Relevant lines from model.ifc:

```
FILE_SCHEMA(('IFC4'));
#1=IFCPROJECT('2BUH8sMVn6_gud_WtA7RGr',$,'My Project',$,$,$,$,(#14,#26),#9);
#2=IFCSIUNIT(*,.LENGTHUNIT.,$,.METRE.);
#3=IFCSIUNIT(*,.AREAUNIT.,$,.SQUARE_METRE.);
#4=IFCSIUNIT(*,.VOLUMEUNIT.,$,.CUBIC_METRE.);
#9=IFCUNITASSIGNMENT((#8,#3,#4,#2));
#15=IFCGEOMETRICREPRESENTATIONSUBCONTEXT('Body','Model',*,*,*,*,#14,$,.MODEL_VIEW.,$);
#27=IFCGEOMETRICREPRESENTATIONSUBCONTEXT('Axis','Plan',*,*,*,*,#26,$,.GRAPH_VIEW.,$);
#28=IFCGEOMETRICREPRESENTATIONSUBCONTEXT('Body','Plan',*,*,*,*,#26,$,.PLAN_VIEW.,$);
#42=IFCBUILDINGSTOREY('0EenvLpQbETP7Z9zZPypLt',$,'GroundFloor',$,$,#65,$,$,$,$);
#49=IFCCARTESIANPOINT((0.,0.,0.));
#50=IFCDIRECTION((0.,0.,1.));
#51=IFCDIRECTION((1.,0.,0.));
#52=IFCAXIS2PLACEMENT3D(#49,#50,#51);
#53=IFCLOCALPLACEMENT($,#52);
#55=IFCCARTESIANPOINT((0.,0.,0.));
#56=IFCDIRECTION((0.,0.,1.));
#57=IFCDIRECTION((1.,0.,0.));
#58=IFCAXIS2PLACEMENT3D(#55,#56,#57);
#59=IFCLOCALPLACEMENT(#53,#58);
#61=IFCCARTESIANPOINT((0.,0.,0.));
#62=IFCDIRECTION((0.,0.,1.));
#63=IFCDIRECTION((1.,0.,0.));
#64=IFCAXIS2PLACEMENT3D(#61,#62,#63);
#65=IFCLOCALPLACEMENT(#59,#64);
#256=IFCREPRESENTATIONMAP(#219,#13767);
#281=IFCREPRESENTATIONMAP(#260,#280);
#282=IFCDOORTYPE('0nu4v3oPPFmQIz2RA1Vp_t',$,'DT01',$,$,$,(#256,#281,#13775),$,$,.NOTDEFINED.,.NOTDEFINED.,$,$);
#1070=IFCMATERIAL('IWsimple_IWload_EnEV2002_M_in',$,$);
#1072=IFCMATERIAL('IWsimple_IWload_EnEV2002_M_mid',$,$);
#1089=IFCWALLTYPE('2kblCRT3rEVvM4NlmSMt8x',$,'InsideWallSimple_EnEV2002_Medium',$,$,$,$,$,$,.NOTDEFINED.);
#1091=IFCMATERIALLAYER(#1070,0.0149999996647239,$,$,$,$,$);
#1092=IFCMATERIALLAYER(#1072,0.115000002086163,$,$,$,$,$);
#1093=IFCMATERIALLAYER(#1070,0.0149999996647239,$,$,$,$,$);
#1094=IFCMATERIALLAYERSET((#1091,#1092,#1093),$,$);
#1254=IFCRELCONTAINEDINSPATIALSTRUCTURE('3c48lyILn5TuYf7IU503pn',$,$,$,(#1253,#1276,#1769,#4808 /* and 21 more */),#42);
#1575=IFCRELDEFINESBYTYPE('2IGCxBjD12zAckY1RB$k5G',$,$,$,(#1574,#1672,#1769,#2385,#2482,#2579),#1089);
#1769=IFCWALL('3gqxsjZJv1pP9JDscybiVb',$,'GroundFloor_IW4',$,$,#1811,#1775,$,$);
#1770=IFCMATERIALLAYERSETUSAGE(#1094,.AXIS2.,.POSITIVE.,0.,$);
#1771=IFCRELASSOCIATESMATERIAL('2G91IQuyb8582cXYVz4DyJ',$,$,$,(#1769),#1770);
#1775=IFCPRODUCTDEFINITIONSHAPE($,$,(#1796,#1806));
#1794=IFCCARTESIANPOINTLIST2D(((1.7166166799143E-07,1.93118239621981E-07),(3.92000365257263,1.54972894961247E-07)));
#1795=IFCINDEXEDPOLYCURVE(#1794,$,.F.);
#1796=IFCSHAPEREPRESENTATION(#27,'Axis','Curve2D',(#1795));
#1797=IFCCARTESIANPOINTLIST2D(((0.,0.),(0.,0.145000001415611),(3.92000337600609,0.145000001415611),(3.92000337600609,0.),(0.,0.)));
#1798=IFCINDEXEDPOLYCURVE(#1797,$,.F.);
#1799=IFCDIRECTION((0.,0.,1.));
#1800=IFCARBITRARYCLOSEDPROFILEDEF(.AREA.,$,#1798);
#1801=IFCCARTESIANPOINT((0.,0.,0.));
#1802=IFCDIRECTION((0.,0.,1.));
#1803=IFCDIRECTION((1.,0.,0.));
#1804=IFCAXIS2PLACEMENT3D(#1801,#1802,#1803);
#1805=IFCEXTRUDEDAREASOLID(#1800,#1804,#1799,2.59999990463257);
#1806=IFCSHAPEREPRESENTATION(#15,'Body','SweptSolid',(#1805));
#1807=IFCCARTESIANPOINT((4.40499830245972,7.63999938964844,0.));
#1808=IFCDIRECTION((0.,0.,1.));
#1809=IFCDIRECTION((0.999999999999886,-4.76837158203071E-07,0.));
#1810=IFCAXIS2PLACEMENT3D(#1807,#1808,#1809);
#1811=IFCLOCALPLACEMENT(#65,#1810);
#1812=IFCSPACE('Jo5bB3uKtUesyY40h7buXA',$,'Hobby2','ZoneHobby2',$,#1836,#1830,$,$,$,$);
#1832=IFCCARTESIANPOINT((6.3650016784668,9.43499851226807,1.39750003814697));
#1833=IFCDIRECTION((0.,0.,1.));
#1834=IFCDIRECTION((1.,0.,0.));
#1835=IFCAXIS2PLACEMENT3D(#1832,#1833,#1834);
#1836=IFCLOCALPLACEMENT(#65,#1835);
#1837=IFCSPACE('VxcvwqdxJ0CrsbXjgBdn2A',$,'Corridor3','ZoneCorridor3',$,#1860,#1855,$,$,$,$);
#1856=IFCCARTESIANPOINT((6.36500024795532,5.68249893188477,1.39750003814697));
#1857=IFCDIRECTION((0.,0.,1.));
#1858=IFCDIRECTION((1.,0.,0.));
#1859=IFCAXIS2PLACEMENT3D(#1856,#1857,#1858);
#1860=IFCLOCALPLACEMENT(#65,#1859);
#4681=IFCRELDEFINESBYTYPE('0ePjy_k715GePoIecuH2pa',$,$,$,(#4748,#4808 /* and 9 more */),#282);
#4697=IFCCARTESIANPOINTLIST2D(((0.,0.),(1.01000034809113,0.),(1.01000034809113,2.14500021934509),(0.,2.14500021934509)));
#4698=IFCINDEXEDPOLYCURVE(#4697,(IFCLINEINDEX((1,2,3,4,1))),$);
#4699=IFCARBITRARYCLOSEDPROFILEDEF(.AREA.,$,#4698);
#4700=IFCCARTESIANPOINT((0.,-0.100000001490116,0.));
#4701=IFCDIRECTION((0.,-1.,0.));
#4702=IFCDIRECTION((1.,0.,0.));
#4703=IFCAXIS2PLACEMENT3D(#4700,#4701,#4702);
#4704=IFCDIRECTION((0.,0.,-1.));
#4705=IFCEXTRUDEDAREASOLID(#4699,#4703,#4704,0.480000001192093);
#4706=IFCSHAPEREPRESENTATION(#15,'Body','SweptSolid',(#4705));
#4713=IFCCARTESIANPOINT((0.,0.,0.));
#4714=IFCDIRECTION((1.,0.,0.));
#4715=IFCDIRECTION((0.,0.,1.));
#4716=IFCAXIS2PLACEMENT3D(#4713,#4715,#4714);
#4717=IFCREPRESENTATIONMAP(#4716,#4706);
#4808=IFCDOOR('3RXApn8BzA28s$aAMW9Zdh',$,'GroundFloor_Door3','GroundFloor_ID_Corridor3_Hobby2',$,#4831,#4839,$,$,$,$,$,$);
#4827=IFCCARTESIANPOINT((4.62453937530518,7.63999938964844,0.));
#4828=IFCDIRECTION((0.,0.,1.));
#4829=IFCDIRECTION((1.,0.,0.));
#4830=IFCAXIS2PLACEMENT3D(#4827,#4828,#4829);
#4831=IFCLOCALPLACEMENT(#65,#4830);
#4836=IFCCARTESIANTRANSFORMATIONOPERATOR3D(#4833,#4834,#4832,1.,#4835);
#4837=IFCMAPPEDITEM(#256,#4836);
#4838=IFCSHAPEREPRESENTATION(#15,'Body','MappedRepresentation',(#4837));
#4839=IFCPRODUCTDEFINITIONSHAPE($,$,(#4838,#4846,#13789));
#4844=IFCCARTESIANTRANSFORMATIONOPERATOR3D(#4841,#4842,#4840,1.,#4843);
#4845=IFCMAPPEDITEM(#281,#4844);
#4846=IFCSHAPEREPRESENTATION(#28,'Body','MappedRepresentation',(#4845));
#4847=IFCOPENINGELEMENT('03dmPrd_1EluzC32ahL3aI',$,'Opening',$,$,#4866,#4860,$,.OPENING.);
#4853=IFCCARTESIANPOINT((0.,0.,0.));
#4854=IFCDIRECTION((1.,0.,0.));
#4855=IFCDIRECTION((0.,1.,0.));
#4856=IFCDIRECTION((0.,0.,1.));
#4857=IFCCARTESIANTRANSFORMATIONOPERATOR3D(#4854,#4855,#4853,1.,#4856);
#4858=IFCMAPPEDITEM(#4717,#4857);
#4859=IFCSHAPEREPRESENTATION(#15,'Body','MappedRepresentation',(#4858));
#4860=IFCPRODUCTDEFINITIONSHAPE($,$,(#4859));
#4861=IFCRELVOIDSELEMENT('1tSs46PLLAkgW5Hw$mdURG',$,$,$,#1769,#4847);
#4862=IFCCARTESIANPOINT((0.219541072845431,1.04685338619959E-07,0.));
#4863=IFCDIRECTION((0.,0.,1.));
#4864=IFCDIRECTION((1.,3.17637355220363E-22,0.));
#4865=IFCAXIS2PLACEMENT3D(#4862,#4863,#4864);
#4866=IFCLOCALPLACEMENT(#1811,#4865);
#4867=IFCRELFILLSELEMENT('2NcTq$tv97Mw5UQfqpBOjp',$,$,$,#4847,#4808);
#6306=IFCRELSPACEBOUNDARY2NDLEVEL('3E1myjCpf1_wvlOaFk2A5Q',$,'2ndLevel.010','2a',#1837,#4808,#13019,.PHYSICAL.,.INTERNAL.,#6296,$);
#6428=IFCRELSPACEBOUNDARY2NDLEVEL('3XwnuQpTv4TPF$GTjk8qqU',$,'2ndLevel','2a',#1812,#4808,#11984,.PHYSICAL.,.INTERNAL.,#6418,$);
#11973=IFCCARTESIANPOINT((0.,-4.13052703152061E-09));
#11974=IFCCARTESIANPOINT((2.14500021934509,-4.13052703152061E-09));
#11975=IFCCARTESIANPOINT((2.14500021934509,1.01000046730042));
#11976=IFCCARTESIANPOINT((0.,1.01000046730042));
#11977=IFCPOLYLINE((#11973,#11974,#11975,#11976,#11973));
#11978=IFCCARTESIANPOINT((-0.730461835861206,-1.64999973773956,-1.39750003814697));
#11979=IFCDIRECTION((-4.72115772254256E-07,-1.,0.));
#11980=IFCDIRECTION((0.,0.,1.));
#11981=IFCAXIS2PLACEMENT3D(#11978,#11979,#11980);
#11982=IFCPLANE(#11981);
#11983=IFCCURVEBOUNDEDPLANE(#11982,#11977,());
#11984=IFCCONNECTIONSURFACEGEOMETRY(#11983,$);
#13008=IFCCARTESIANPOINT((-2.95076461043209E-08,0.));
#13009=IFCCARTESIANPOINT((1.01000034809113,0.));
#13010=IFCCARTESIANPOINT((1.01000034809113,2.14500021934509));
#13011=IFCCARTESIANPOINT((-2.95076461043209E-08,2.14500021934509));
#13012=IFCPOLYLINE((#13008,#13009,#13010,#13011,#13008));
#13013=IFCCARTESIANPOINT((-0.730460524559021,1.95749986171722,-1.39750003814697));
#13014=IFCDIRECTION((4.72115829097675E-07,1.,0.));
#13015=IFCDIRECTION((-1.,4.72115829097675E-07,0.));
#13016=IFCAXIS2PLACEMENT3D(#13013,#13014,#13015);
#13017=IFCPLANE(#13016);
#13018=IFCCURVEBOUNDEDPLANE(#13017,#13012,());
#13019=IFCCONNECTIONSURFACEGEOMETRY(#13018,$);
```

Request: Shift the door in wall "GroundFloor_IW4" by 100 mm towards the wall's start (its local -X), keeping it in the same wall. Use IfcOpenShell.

```python
import numpy as np
import ifcopenshell
import ifcopenshell.api.geometry
import ifcopenshell.util.placement

model = ifcopenshell.open("model.ifc")

door = model.by_id(4808)
opening = door.FillsVoids[0].RelatingOpeningElement
wall = opening.VoidsElements[0].RelatingBuildingElement

wall_matrix = ifcopenshell.util.placement.get_local_placement(wall.ObjectPlacement)
shift = wall_matrix[:3, 0] * -0.1
before = ifcopenshell.util.placement.get_local_placement(door.ObjectPlacement)[:3, 3].copy()

# The door is not placed relative to its opening, so move both.
for product in (opening, door):
    matrix = ifcopenshell.util.placement.get_local_placement(product.ObjectPlacement)
    matrix[:3, 3] += shift
    ifcopenshell.api.geometry.edit_object_placement(model, product=product, matrix=matrix, is_si=False)

# Space boundary surfaces are stored in each space's coordinates; move them too.
for rel in door.ProvidesBoundaries:
    if not rel.ConnectionGeometry:
        continue
    surface = rel.ConnectionGeometry.SurfaceOnRelatingElement.BasisSurface
    space_matrix = ifcopenshell.util.placement.get_local_placement(rel.RelatingSpace.ObjectPlacement)
    point = np.array(surface.Position.Location.Coordinates) + space_matrix[:3, :3].T @ shift
    surface.Position = model.createIfcAxis2Placement3D(
        model.createIfcCartesianPoint(point.tolist()), surface.Position.Axis, surface.Position.RefDirection
    )

after = ifcopenshell.util.placement.get_local_placement(door.ObjectPlacement)[:3, 3]
print("door moved by", (after - before).round(3) + 0.0)

model.write("model_v2.ifc")
```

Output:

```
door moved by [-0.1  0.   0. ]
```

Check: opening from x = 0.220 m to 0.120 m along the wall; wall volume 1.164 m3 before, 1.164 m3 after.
